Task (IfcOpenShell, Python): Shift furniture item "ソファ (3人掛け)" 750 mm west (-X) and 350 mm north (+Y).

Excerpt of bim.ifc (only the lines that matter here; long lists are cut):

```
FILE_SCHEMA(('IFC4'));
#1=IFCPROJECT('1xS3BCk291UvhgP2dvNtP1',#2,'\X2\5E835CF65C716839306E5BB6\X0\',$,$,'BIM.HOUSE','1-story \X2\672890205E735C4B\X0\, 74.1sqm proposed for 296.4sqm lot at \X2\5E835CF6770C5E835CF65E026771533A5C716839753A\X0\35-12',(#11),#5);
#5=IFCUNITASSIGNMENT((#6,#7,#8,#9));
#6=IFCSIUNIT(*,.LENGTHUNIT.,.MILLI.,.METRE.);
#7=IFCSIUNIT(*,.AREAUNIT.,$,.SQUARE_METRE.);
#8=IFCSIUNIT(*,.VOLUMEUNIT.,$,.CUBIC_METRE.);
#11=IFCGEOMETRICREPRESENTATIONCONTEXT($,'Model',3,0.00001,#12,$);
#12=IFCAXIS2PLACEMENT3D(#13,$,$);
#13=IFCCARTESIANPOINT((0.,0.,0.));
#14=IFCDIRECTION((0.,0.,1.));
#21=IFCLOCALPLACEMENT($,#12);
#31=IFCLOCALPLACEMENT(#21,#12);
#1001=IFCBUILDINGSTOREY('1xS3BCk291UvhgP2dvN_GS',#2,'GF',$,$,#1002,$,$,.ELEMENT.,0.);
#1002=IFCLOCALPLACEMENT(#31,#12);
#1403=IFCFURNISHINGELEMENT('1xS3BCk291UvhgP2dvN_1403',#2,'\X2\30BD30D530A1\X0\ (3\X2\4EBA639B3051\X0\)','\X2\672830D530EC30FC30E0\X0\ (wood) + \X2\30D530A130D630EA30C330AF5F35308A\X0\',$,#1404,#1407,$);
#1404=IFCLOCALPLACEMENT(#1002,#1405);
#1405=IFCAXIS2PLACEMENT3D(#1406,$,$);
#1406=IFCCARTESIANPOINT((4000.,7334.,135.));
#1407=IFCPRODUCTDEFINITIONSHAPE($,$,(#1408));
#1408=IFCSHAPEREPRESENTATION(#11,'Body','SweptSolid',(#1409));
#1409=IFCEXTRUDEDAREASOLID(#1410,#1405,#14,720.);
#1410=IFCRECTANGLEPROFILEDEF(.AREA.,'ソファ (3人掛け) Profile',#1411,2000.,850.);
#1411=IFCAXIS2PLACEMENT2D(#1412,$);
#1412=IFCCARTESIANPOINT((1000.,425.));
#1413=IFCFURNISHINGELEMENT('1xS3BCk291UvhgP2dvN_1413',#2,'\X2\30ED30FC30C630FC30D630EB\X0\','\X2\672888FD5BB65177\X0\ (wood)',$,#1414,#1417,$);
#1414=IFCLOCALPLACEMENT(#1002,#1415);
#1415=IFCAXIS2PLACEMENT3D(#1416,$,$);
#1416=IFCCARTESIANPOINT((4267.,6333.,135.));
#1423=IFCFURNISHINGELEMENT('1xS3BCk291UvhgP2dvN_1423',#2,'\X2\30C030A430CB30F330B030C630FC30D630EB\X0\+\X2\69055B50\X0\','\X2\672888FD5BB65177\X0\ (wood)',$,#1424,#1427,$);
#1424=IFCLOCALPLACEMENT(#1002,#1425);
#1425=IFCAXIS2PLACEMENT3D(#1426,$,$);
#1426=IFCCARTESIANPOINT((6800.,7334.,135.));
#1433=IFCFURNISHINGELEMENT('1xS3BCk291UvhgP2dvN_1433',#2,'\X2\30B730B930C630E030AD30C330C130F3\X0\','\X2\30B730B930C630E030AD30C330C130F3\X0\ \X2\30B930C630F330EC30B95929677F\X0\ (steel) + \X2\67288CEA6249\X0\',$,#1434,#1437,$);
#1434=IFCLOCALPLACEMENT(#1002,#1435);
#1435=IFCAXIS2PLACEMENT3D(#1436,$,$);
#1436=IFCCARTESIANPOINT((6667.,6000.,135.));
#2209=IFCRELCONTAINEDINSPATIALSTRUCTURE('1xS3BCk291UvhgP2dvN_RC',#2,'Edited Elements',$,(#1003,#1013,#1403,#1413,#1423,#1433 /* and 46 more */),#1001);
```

```python
import ifcopenshell
import ifcopenshell.api.geometry
import ifcopenshell.util.placement
import ifcopenshell.util.unit

model = ifcopenshell.open("bim.ifc")
unit_scale = ifcopenshell.util.unit.calculate_unit_scale(model)

item = model.by_guid("1xS3BCk291UvhgP2dvN_1403")
matrix = ifcopenshell.util.placement.get_local_placement(item.ObjectPlacement)
matrix[0, 3] -= 0.75 / unit_scale
matrix[1, 3] += 0.35 / unit_scale
ifcopenshell.api.geometry.edit_object_placement(model, product=item, matrix=matrix, is_si=False)

print(ifcopenshell.util.placement.get_local_placement(item.ObjectPlacement).round(3) + 0.0)

model.write("bim_rev.ifc")
```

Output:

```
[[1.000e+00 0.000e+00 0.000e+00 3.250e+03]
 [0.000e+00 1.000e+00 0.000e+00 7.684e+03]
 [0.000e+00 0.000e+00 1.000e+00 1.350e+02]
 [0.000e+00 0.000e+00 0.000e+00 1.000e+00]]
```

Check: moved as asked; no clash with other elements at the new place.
